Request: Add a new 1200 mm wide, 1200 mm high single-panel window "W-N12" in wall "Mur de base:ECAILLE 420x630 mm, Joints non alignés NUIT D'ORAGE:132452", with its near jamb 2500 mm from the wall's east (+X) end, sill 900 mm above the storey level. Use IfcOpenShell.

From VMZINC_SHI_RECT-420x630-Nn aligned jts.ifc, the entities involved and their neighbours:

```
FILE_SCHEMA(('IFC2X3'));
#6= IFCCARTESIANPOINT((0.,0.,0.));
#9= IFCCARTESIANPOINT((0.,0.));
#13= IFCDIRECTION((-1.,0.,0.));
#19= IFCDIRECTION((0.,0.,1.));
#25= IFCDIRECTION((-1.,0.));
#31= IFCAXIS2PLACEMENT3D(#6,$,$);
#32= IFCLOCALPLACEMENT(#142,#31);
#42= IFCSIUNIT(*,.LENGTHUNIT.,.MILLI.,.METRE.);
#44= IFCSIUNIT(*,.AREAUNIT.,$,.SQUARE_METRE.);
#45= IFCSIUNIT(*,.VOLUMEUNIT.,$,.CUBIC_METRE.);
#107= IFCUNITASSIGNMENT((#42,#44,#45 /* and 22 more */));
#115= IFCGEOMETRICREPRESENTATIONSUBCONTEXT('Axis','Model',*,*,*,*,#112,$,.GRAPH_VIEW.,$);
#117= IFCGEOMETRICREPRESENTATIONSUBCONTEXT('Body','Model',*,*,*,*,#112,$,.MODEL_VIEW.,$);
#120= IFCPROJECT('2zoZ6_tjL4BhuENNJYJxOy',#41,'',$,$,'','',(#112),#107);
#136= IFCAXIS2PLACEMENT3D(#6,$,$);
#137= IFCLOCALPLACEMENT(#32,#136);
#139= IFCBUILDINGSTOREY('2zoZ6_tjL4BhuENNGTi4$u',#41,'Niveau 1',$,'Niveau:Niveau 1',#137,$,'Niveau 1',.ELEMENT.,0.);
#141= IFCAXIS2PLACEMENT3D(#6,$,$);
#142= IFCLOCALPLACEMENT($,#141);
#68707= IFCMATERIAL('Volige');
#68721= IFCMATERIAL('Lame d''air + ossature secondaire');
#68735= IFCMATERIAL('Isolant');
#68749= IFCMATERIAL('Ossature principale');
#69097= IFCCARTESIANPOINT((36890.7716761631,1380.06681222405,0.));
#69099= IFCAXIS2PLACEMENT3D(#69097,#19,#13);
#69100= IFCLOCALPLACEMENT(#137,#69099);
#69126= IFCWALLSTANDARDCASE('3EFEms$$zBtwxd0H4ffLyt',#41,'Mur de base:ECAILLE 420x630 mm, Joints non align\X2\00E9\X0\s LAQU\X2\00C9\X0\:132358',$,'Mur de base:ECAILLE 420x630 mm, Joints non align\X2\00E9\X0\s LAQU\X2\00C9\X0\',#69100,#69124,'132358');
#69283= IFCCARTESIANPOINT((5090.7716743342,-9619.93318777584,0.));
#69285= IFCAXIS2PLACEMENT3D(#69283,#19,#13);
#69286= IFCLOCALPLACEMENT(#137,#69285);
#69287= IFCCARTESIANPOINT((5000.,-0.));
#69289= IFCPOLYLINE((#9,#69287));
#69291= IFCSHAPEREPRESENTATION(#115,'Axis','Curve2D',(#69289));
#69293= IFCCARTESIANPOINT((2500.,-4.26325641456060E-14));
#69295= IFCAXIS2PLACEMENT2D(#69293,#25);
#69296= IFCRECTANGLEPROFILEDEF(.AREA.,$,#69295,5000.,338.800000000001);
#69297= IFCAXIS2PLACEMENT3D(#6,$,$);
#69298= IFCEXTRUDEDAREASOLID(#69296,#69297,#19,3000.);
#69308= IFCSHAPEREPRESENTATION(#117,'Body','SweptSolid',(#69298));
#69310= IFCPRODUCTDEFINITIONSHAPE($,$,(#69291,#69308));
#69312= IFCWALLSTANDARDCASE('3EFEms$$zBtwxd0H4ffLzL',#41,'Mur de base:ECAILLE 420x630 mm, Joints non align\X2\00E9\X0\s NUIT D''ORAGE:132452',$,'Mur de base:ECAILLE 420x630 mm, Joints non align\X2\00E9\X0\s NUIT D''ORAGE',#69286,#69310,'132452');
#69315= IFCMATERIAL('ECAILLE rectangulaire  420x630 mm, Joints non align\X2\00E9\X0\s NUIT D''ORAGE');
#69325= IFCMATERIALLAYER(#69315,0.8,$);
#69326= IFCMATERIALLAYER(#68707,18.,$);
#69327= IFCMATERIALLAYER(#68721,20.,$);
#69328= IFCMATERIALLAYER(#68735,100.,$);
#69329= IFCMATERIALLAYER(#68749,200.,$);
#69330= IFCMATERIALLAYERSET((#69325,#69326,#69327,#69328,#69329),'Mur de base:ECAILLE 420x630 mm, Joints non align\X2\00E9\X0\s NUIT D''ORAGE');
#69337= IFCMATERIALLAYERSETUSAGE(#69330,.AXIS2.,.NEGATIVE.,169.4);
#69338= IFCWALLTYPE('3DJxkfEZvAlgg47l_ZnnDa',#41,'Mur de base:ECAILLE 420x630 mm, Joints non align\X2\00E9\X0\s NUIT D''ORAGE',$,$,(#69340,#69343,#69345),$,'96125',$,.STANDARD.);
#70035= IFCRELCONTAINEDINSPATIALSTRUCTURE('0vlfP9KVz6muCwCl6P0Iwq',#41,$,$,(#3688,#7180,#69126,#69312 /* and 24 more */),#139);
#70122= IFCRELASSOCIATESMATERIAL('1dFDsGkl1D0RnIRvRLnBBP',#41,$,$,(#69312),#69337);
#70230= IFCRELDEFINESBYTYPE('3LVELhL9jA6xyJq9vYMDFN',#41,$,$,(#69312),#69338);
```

```python
import numpy as np
import ifcopenshell
import ifcopenshell.api.feature
import ifcopenshell.api.geometry
import ifcopenshell.api.root
import ifcopenshell.api.spatial
import ifcopenshell.api.type
import ifcopenshell.geom
import ifcopenshell.util.element
import ifcopenshell.util.placement
import ifcopenshell.util.representation
import ifcopenshell.util.shape
import ifcopenshell.util.unit

model = ifcopenshell.open("VMZINC_SHI_RECT-420x630-Nn aligned jts.ifc")
unit_scale = ifcopenshell.util.unit.calculate_unit_scale(model)
settings = ifcopenshell.geom.settings()


def volume(element):
    """Net volume in cubic metres, openings subtracted."""
    shape = ifcopenshell.geom.create_shape(settings, element)
    return ifcopenshell.util.shape.get_volume(shape.geometry)


wall = model.by_guid("3EFEms$$zBtwxd0H4ffLzL")
storey = ifcopenshell.util.element.get_container(wall, ifc_class="IfcBuildingStorey")
context = ifcopenshell.util.representation.get_context(model, "Model", "Body", "MODEL_VIEW")
before = volume(wall)

width, height, from_end, sill = 1.2, 1.2, 2.5, 0.9  # metres

# The wall runs along its own X axis, and the end named is its -X end.
wall_shape = ifcopenshell.geom.create_shape(settings, wall)
x, y, z = ifcopenshell.util.shape.get_vertices(wall_shape.geometry).T
start = x.min() + from_end
face, thickness = float(y.min()), float(y.max() - y.min())
wall_matrix = ifcopenshell.util.placement.get_local_placement(wall.ObjectPlacement)
level = ifcopenshell.util.placement.get_local_placement(storey.ObjectPlacement)[2, 3]


def in_wall(x, y):
    """Placement at x, y metres in the wall's axes, at sill height."""
    matrix = wall_matrix.copy()
    matrix[:, 3] = wall_matrix @ np.array([x / unit_scale, y / unit_scale, 0.0, 1.0])
    matrix[2, 3] = level + sill / unit_scale
    return matrix


# Opening: a box that overshoots both wall faces by 50 mm.
opening = ifcopenshell.api.root.create_entity(model, ifc_class="IfcOpeningElement")
box = ifcopenshell.api.geometry.add_wall_representation(
    model, context=context, length=width, height=height, thickness=thickness + 0.1
)
ifcopenshell.api.geometry.assign_representation(model, product=opening, representation=box)
ifcopenshell.api.geometry.edit_object_placement(model, product=opening, matrix=in_wall(start, face - 0.05), is_si=False)
ifcopenshell.api.feature.add_feature(model, feature=opening, element=wall)

window = ifcopenshell.api.root.create_entity(model, ifc_class="IfcWindow", name="W-N12")
window.OverallWidth, window.OverallHeight = width / unit_scale, height / unit_scale
body = ifcopenshell.api.geometry.add_window_representation(
    model,
    context=context,
    overall_width=window.OverallWidth,
    overall_height=window.OverallHeight,
    partition_type="SINGLE_PANEL",
)
ifcopenshell.api.geometry.assign_representation(model, product=window, representation=body)
ifcopenshell.api.spatial.assign_container(model, products=[window], relating_structure=storey)
fills = ifcopenshell.api.feature.add_filling(model, opening=opening, element=window)
fills.OwnerHistory = window.OwnerHistory  # required in IFC2X3

# IFC2X3 keeps the operation on the window style.
style = ifcopenshell.api.root.create_entity(model, ifc_class="IfcWindowStyle", name="W-N12")
style.OperationType, style.ConstructionType = "SINGLE_PANEL", "NOTDEFINED"
style.ParameterTakesPrecedence = style.Sizeable = False
ifcopenshell.api.type.assign_type(model, related_objects=[window], relating_type=style)

# Centre the window in the wall's thickness.
ifcopenshell.api.geometry.edit_object_placement(model, product=window, matrix=in_wall(start, face), is_si=False)
window_shape = ifcopenshell.geom.create_shape(settings, window)
depth = ifcopenshell.util.shape.get_vertices(window_shape.geometry)[:, 1]
offset = face + thickness / 2 - (depth.min() + depth.max()) / 2
ifcopenshell.api.geometry.edit_object_placement(model, product=window, matrix=in_wall(start, offset), is_si=False)

after = volume(wall)

print(f"wall volume {before:.3f} -> {after:.3f} m3")

model.write("VMZINC_SHI_RECT-420x630-Nn aligned jts_v2.ifc")
```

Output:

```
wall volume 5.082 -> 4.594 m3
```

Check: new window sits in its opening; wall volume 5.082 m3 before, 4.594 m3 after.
